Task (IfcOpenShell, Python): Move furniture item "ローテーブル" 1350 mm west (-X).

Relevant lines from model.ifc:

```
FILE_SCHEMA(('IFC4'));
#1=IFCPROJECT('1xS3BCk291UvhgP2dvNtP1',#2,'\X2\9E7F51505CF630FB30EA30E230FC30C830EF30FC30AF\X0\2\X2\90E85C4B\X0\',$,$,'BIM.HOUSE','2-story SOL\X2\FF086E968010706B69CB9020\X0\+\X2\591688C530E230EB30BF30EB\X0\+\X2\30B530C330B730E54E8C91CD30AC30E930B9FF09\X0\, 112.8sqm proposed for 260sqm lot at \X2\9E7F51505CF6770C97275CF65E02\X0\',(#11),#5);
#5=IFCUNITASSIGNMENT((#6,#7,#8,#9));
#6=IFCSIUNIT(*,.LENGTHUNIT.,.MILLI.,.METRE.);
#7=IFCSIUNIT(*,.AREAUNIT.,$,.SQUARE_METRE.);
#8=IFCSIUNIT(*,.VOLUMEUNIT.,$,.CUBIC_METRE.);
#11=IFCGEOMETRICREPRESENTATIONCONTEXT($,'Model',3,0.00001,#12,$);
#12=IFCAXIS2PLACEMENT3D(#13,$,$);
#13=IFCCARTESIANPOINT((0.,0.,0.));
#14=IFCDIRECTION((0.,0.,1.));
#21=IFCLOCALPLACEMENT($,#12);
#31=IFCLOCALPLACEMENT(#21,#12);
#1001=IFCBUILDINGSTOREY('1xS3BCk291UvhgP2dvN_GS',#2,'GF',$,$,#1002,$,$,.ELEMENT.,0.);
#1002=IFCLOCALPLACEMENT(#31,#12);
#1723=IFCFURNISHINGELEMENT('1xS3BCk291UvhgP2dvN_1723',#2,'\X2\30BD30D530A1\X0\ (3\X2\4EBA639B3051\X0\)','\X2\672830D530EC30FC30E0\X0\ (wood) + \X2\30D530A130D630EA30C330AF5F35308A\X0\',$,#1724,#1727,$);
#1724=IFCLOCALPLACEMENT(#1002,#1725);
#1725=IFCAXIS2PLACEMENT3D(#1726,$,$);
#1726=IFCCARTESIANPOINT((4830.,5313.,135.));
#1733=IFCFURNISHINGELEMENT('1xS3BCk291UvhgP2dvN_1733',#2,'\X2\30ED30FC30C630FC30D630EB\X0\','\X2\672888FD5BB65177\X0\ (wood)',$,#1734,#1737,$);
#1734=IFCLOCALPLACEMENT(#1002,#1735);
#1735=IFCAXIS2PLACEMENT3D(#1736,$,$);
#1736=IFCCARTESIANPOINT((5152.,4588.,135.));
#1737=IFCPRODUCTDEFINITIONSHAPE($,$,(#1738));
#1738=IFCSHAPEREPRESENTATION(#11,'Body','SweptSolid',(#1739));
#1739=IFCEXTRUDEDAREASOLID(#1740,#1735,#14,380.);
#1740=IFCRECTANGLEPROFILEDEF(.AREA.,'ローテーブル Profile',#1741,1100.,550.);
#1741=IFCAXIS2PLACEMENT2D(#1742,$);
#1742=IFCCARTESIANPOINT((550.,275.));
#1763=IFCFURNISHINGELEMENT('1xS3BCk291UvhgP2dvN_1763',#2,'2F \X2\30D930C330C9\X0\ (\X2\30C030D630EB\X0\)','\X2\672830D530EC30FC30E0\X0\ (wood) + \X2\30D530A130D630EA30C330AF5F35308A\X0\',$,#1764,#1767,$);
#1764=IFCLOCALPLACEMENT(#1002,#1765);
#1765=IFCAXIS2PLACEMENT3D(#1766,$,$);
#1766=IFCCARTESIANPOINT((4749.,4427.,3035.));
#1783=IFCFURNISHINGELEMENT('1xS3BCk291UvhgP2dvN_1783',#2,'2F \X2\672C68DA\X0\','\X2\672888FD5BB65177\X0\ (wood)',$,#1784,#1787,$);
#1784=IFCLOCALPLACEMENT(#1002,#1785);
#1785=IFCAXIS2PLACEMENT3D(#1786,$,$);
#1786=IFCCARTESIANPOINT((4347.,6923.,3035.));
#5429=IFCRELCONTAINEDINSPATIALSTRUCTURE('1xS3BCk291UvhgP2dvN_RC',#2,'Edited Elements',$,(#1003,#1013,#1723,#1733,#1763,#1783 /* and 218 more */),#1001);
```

```python
import ifcopenshell
import ifcopenshell.api.geometry
import ifcopenshell.util.placement
import ifcopenshell.util.unit

model = ifcopenshell.open("model.ifc")
unit_scale = ifcopenshell.util.unit.calculate_unit_scale(model)

item = model.by_guid("1xS3BCk291UvhgP2dvN_1733")
matrix = ifcopenshell.util.placement.get_local_placement(item.ObjectPlacement)
matrix[0, 3] -= 1.35 / unit_scale
ifcopenshell.api.geometry.edit_object_placement(model, product=item, matrix=matrix, is_si=False)

print(ifcopenshell.util.placement.get_local_placement(item.ObjectPlacement).round(3) + 0.0)

model.write("model_updated.ifc")
```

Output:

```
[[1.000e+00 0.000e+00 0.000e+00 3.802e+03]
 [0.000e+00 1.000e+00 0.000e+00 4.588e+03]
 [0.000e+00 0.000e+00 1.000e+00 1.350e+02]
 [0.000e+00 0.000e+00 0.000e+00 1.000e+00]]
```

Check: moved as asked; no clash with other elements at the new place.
